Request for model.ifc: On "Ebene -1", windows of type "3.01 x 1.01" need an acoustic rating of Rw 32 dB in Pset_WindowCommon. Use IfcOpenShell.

First a look at what the model holds.

```python
import ifcopenshell
import ifcopenshell.util.element

model = ifcopenshell.open("model.ifc")
print(model.schema)
storey = next(s for s in model.by_type("IfcBuildingStorey") if s.Name == "Ebene -1")
windows = [e for e in ifcopenshell.util.element.get_decomposition(storey) if e.is_a("IfcWindow")]
seen = {}
for e in windows:
    element_type = ifcopenshell.util.element.get_type(e)
    key = (element_type.Name if element_type != e and element_type else None, ifcopenshell.util.element.get_pset(e, "Pset_WindowCommon", "AcousticRating"))
    seen[key] = seen.get(key, 0) + 1
for (name, value), count in sorted(seen.items(), key=str):
    print(count, "x", name, "|", value)
```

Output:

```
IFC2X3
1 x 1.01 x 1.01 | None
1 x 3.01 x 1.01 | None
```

```python
import ifcopenshell
import ifcopenshell.api.pset
import ifcopenshell.util.element

model = ifcopenshell.open("model.ifc")

storey = next(s for s in model.by_type("IfcBuildingStorey") if s.Name == "Ebene -1")
windows = [e for e in ifcopenshell.util.element.get_decomposition(storey) if e.is_a("IfcWindow")]

count = 0
for e in windows:
    element_type = ifcopenshell.util.element.get_type(e)
    if element_type in (None, e) or element_type.Name != "3.01 x 1.01":
        continue
    # add_pset returns the element's existing set when there is one.
    pset = ifcopenshell.api.pset.add_pset(model, product=e, name="Pset_WindowCommon")
    ifcopenshell.api.pset.edit_pset(model, pset=pset, properties={"AcousticRating": "Rw 32 dB"})
    count += 1

print(count, "windows updated")

model.write("model-out.ifc")
```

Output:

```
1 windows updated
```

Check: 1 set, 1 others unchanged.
